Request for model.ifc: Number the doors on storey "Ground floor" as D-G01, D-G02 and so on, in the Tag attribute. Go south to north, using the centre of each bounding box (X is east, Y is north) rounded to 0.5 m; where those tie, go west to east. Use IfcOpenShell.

First a look at what the model holds.

```python
import ifcopenshell
import ifcopenshell.util.element
import ifcopenshell.util.placement

model = ifcopenshell.open("model.ifc")
print(model.schema)
storey = next(s for s in model.by_type("IfcBuildingStorey") if s.Name == "Ground floor")
doors = [e for e in ifcopenshell.util.element.get_decomposition(storey) if e.is_a("IfcDoor")]
for e in sorted(doors, key=lambda e: e.id()):
    origin = ifcopenshell.util.placement.get_local_placement(e.ObjectPlacement)[:3, 3]
    print(e.id(), e.Tag, e.Name, origin.round(2) + 0.0, sep=" | ")
```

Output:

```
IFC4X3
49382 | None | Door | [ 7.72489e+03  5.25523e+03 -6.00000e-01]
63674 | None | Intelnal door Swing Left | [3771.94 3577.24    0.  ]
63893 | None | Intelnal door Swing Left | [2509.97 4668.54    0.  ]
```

```python
import ifcopenshell
import ifcopenshell.geom
import ifcopenshell.util.element
import ifcopenshell.util.shape

model = ifcopenshell.open("model.ifc")
settings = ifcopenshell.geom.settings()
settings.set("use-world-coords", True)


def centre(element):
    shape = ifcopenshell.geom.create_shape(settings, element)
    return ifcopenshell.util.shape.get_bbox_centroid(shape.geometry)


storey = next(s for s in model.by_type("IfcBuildingStorey") if s.Name == "Ground floor")
doors = [e for e in ifcopenshell.util.element.get_decomposition(storey) if e.is_a("IfcDoor")]

# Insertion points can sit at a corner or the storey origin, so sort by the geometry (in metres).
centres = {e: centre(e) for e in doors}
doors.sort(key=lambda e: (round(centres[e][1] / 0.5), centres[e][0]))

for i, e in enumerate(doors, start=1):
    number = f"D-G{i:02d}"
    e.Tag = number
    print(e.id(), number)

model.write("model-out.ifc")
```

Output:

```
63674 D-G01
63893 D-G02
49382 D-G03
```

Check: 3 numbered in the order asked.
